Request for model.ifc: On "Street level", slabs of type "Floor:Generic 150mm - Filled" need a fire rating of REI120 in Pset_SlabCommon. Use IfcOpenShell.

First a look at what the model holds.

```python
import ifcopenshell
import ifcopenshell.util.element

model = ifcopenshell.open("model.ifc")
print(model.schema)
storey = next(s for s in model.by_type("IfcBuildingStorey") if s.Name == "Street level")
slabs = [e for e in ifcopenshell.util.element.get_decomposition(storey) if e.is_a("IfcSlab")]
seen = {}
for e in slabs:
    element_type = ifcopenshell.util.element.get_type(e)
    key = (element_type.Name if element_type != e and element_type else None, ifcopenshell.util.element.get_pset(e, "Pset_SlabCommon", "FireRating"))
    seen[key] = seen.get(key, 0) + 1
for (name, value), count in sorted(seen.items(), key=str):
    print(count, "x", name, "|", value)
```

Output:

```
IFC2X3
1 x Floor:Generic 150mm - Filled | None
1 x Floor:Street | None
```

```python
import ifcopenshell
import ifcopenshell.api.pset
import ifcopenshell.util.element

model = ifcopenshell.open("model.ifc")

storey = next(s for s in model.by_type("IfcBuildingStorey") if s.Name == "Street level")
slabs = [e for e in ifcopenshell.util.element.get_decomposition(storey) if e.is_a("IfcSlab")]

count = 0
for e in slabs:
    element_type = ifcopenshell.util.element.get_type(e)
    if element_type in (None, e) or element_type.Name != "Floor:Generic 150mm - Filled":
        continue
    # add_pset returns the element's existing set when there is one.
    pset = ifcopenshell.api.pset.add_pset(model, product=e, name="Pset_SlabCommon")
    ifcopenshell.api.pset.edit_pset(model, pset=pset, properties={"FireRating": "REI120"})
    count += 1

print(count, "slabs updated")

model.write("model_rev.ifc")
```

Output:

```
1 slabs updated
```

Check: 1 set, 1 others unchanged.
